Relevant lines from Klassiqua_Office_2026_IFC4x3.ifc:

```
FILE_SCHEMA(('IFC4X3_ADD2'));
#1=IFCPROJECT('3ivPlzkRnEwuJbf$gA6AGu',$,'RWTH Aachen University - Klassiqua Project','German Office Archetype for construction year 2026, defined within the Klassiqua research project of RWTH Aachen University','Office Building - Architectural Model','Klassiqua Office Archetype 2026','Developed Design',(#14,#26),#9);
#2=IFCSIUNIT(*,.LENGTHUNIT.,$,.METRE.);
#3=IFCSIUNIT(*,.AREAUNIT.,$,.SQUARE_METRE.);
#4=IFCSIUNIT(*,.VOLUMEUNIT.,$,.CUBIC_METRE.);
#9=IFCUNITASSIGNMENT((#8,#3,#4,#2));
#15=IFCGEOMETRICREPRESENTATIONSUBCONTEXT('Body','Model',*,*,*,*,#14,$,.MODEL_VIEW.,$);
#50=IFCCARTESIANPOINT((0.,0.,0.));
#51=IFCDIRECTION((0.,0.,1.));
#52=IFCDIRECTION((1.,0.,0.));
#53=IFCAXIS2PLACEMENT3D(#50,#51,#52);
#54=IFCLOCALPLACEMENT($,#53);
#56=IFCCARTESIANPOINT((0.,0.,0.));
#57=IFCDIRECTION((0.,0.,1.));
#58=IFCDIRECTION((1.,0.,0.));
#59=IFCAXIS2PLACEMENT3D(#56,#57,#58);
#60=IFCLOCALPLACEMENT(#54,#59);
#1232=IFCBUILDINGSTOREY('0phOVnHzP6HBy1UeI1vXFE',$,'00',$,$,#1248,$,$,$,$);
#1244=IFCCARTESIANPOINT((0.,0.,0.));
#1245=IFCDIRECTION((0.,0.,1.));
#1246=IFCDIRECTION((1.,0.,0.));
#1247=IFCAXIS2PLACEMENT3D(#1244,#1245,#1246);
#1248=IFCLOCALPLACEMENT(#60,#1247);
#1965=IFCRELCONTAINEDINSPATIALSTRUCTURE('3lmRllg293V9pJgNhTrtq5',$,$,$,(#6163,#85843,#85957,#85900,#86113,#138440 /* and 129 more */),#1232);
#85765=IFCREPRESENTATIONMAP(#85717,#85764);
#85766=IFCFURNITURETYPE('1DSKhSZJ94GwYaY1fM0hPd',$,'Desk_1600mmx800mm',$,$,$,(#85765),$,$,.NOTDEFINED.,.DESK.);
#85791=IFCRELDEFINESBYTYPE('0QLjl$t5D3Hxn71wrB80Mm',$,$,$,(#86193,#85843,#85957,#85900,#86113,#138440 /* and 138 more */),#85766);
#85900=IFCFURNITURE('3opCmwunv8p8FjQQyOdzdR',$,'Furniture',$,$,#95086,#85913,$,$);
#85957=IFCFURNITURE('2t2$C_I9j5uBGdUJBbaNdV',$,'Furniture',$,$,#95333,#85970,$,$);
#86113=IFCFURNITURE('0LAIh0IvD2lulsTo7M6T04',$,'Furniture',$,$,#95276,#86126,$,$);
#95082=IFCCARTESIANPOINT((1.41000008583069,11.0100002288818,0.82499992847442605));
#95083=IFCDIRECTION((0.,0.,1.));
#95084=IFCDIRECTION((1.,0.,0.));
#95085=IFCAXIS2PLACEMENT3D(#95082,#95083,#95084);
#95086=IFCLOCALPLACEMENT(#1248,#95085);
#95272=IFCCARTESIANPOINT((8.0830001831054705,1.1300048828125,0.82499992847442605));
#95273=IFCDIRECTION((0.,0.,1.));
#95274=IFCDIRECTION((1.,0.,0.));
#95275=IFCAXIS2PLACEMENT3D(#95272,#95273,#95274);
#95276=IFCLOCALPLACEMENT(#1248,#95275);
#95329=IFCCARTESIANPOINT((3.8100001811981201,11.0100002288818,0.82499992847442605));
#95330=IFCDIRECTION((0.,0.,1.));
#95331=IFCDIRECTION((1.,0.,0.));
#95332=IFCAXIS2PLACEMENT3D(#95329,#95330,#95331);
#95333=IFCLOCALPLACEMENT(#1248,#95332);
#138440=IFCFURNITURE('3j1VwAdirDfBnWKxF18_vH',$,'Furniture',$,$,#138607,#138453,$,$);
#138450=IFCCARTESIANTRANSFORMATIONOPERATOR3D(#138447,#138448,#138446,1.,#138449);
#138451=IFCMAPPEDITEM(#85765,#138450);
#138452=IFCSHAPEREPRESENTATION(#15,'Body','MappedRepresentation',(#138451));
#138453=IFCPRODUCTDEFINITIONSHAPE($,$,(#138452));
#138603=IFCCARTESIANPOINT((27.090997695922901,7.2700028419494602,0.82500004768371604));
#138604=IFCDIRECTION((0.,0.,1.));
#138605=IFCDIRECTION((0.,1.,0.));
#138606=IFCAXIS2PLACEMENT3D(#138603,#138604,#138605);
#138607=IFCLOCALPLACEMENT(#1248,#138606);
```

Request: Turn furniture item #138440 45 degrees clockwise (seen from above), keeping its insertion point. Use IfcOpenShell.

```python
import ifcopenshell
import ifcopenshell.api.geometry
import ifcopenshell.util.placement

model = ifcopenshell.open("Klassiqua_Office_2026_IFC4x3.ifc")

item = model.by_guid("3j1VwAdirDfBnWKxF18_vH")
matrix = ifcopenshell.util.placement.get_local_placement(item.ObjectPlacement)
matrix = matrix @ ifcopenshell.util.placement.rotation(-45, "Z")
ifcopenshell.api.geometry.edit_object_placement(model, product=item, matrix=matrix, is_si=False)

print(ifcopenshell.util.placement.get_local_placement(item.ObjectPlacement).round(3) + 0.0)

model.write("Klassiqua_Office_2026_IFC4x3-out.ifc")
```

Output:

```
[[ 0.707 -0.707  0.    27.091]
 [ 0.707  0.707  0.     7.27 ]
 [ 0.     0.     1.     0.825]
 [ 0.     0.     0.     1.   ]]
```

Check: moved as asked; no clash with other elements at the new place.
